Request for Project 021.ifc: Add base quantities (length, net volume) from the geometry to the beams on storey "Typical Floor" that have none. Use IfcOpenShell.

First a look at what the model holds.

```python
import ifcopenshell
import ifcopenshell.util.element
import ifcopenshell.util.unit

model = ifcopenshell.open("Project 021.ifc")
print(model.schema)
for unit_type in ("LENGTHUNIT", "AREAUNIT", "VOLUMEUNIT"):
    print(unit_type, ifcopenshell.util.unit.calculate_unit_scale(model, unit_type))
storey = next(s for s in model.by_type("IfcBuildingStorey") if s.Name == "Typical Floor")
beams = [e for e in ifcopenshell.util.element.get_decomposition(storey) if e.is_a("IfcBeam")]
for e in sorted(beams, key=lambda e: e.id()):
    print(e.id(), e.is_a(), e.Name, list(ifcopenshell.util.element.get_psets(e, qtos_only=True)), sep=" | ")
```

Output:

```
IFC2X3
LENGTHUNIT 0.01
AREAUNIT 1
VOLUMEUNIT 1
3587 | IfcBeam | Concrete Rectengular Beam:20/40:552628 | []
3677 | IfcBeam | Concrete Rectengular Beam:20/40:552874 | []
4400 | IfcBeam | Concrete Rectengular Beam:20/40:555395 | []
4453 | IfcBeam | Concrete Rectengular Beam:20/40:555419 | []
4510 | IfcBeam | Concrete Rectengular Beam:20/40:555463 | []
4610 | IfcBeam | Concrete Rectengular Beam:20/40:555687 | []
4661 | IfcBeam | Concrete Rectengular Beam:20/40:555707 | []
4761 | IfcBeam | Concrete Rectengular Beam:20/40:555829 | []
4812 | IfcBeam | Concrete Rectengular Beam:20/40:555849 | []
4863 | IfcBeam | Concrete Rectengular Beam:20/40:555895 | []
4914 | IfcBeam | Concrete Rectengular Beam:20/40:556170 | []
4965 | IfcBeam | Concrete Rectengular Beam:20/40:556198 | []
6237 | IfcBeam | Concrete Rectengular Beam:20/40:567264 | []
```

```python
import ifcopenshell
import ifcopenshell.api.pset
import ifcopenshell.geom
import ifcopenshell.util.element
import ifcopenshell.util.shape
import ifcopenshell.util.unit

model = ifcopenshell.open("Project 021.ifc")
unit_scale = ifcopenshell.util.unit.calculate_unit_scale(model)
volume_scale = ifcopenshell.util.unit.calculate_unit_scale(model, "VOLUMEUNIT")
settings = ifcopenshell.geom.settings()

storey = next(s for s in model.by_type("IfcBuildingStorey") if s.Name == "Typical Floor")
beams = [e for e in ifcopenshell.util.element.get_decomposition(storey) if e.is_a("IfcBeam")]

for e in sorted(beams, key=lambda e: e.id()):
    if ifcopenshell.util.element.get_psets(e, qtos_only=True, should_inherit=False):
        continue
    # Geometry comes back in metres, in the element's own axes.
    shape = ifcopenshell.geom.create_shape(settings, e)
    values = {
        "Length": ifcopenshell.util.shape.get_max_xyz(shape.geometry) / unit_scale,
        "NetVolume": ifcopenshell.util.shape.get_volume(shape.geometry) / volume_scale,
    }
    qto = ifcopenshell.api.pset.add_qto(model, product=e, name="BaseQuantities")
    ifcopenshell.api.pset.edit_qto(model, qto=qto, properties=values)
    print(e.id(), {k: round(v, 3) for k, v in values.items()})

model.write("Project 021_updated.ifc")
```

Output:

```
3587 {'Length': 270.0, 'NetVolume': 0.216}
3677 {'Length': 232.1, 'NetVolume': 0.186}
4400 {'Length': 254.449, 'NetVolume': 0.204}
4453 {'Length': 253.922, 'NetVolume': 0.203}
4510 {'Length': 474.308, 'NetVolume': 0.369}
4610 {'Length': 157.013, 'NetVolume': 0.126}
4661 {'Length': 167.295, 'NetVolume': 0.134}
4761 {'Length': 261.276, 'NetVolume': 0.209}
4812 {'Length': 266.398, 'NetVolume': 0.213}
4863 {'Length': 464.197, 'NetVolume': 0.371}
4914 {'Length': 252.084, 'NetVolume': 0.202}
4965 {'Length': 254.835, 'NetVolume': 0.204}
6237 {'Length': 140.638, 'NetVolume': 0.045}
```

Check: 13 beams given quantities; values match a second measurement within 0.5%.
